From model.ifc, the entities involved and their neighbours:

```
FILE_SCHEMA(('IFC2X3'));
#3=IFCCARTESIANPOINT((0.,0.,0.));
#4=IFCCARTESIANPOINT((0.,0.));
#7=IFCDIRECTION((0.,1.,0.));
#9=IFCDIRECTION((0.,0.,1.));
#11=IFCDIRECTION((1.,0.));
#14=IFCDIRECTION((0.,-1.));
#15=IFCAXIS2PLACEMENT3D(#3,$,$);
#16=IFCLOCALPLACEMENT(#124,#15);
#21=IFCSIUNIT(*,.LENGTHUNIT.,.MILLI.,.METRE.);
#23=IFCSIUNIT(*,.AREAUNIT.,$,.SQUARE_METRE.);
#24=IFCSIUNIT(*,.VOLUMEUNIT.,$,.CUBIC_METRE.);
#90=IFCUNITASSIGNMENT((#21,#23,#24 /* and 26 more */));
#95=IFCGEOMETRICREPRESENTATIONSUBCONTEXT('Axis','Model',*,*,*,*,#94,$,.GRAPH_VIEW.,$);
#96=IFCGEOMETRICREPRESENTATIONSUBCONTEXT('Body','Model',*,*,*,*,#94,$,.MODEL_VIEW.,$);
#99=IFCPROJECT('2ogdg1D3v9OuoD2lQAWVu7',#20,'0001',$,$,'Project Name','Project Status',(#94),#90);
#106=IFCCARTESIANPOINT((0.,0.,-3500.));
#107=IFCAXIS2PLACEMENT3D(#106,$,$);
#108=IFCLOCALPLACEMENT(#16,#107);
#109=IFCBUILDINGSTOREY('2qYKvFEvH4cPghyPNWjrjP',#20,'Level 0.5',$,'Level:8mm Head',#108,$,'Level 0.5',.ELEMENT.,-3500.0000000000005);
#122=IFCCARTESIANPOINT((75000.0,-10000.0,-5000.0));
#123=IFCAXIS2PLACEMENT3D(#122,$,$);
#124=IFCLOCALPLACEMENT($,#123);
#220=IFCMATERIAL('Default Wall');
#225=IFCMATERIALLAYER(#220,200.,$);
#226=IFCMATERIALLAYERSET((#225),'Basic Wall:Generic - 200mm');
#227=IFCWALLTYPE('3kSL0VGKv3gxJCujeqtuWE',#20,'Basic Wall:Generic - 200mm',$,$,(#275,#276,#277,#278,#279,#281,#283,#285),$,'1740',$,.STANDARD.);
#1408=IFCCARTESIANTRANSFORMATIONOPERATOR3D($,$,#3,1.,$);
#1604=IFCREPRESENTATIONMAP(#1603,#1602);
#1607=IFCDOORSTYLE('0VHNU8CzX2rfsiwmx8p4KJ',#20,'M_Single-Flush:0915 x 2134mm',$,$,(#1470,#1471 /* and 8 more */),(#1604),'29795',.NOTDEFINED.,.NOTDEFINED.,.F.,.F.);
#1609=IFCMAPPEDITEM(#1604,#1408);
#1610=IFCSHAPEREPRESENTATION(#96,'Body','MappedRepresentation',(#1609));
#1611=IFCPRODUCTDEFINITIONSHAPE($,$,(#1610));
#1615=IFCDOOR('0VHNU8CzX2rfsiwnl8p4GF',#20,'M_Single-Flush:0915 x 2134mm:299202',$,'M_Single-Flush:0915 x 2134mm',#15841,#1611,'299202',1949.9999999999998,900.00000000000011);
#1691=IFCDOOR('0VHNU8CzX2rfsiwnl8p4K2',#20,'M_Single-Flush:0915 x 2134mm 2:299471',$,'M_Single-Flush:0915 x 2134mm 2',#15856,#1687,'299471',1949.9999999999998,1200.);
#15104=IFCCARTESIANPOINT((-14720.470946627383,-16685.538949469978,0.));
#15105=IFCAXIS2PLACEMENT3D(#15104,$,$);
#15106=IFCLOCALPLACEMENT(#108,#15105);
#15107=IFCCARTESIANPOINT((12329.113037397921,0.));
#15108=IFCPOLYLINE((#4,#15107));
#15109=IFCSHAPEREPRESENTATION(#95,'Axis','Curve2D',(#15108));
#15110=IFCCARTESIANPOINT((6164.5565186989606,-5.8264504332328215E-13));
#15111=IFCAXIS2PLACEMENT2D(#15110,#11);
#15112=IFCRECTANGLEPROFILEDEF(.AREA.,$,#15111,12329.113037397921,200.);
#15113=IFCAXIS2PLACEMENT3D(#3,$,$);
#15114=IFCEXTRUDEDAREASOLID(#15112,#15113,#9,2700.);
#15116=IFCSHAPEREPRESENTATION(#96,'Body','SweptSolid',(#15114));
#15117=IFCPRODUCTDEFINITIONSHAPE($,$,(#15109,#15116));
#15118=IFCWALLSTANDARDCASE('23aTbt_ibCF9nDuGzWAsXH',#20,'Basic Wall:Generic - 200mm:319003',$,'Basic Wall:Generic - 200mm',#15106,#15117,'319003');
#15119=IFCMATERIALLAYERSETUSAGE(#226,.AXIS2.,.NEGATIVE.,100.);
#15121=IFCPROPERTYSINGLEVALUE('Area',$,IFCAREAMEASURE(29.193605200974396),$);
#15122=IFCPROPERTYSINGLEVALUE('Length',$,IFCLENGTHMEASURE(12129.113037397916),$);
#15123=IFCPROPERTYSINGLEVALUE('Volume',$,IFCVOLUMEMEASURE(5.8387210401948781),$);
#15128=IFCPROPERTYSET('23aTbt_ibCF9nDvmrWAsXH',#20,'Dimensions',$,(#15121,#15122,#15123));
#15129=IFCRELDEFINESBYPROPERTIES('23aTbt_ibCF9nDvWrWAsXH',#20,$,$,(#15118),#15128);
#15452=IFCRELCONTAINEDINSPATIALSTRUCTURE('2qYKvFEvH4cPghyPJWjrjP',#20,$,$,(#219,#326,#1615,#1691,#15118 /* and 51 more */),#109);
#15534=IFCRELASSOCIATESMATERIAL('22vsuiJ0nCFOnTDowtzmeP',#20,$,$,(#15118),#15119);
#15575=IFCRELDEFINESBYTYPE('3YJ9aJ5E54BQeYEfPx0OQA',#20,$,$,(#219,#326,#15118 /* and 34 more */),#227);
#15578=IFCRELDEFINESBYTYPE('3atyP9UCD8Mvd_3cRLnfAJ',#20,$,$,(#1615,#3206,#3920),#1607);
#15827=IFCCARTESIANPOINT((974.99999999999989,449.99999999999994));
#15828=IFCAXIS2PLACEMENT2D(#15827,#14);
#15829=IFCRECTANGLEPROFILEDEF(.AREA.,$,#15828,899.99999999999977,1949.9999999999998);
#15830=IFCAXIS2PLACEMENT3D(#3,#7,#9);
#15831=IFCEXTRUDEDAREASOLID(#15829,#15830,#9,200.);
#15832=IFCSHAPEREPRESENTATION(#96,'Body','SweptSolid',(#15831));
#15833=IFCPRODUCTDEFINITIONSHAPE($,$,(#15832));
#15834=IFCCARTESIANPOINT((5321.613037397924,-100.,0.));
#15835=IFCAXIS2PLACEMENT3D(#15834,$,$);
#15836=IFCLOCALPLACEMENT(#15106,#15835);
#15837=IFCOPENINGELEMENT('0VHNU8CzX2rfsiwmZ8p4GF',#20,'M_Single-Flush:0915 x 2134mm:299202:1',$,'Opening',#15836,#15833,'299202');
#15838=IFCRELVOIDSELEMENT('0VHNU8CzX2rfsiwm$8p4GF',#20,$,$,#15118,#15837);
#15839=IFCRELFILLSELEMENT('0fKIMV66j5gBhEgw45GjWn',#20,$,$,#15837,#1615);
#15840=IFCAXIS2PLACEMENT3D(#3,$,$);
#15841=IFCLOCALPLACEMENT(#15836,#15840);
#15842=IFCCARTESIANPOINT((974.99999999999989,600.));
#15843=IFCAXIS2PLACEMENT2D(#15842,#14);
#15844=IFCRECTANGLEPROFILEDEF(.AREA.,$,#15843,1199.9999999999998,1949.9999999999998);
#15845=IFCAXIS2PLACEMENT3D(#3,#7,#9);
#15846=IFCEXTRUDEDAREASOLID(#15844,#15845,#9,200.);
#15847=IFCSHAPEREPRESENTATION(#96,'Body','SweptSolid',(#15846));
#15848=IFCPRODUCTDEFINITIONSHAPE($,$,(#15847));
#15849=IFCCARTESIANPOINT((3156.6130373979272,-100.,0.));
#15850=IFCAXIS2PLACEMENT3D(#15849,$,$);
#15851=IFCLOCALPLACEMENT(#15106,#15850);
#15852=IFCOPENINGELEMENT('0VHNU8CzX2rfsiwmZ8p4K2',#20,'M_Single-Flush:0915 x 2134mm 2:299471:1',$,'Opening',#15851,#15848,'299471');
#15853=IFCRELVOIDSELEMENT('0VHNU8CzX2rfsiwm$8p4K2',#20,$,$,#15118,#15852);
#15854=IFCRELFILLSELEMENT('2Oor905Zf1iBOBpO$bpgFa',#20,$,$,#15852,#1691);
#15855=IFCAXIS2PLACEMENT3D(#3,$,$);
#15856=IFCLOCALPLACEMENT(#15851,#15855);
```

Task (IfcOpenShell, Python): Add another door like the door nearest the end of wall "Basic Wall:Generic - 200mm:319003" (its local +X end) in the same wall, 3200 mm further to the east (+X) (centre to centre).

```python
import ifcopenshell
import ifcopenshell.api.feature
import ifcopenshell.api.geometry
import ifcopenshell.api.pset
import ifcopenshell.api.root
import ifcopenshell.geom
import ifcopenshell.util.element
import ifcopenshell.util.placement
import ifcopenshell.util.shape
import ifcopenshell.util.unit

model = ifcopenshell.open("model.ifc")
unit_scale = ifcopenshell.util.unit.calculate_unit_scale(model)
area_scale = ifcopenshell.util.unit.calculate_unit_scale(model, "AREAUNIT")
volume_scale = ifcopenshell.util.unit.calculate_unit_scale(model, "VOLUMEUNIT")
settings = ifcopenshell.geom.settings()


def volume(element):
    """Net volume in cubic metres, openings subtracted."""
    shape = ifcopenshell.geom.create_shape(settings, element)
    return ifcopenshell.util.shape.get_volume(shape.geometry)


def reuse_history(source, copy):
    """copy_class also copies each property set's owner history, people and application; keep the originals."""
    for rel in copy.IsDefinedBy:
        if rel.is_a("IfcRelDefinesByProperties") and (history := rel.RelatingPropertyDefinition.OwnerHistory):
            rel.RelatingPropertyDefinition.OwnerHistory = source.OwnerHistory
            ifcopenshell.util.element.remove_deep2(model, history)


door = model.by_guid("0VHNU8CzX2rfsiwnl8p4GF")
opening = door.FillsVoids[0].RelatingOpeningElement
wall = opening.VoidsElements[0].RelatingBuildingElement
before = volume(wall)
shift = ifcopenshell.util.placement.get_local_placement(wall.ObjectPlacement)[:3, 0] * 3.2 / unit_scale

# copy_class copies the void relationship, type, container and properties, but no geometry.
new_opening = ifcopenshell.api.root.copy_class(model, product=opening)
new_opening.Representation = ifcopenshell.util.element.copy_deep(
    model, opening.Representation, exclude=["IfcGeometricRepresentationContext", "IfcRepresentationMap"]
)
new_opening.Name = "M_Single-Flush:0915 x 2134mm"
new_opening.Tag = None
new_door = ifcopenshell.api.root.copy_class(model, product=door)
new_door.Representation = ifcopenshell.util.element.copy_deep(
    model, door.Representation, exclude=["IfcGeometricRepresentationContext", "IfcRepresentationMap"]
)
new_door.Name = "M_Single-Flush:0915 x 2134mm"
new_door.Tag = None
reuse_history(door, new_door)
fills = ifcopenshell.api.feature.add_filling(model, opening=new_opening, element=new_door)
fills.OwnerHistory = new_door.OwnerHistory  # required in IFC2X3

for old, new in ((opening, new_opening), (door, new_door)):
    matrix = ifcopenshell.util.placement.get_local_placement(old.ObjectPlacement)
    matrix[:3, 3] += shift
    ifcopenshell.api.geometry.edit_object_placement(model, product=new, matrix=matrix, is_si=False)

after = volume(wall)
thickness = 0.2  # wall thickness in metres

# Update the wall's stored quantities.
pset = model.by_id(ifcopenshell.util.element.get_pset(wall, "Dimensions", should_inherit=False)["id"])
ifcopenshell.api.pset.edit_pset(model, pset=pset, properties={
    "Area": model.create_entity("IfcAreaMeasure", after / thickness / area_scale),
    "Volume": model.create_entity("IfcVolumeMeasure", after / volume_scale),
})

print(f"wall volume {before:.3f} -> {after:.3f} m3")

model.write("model-out.ifc")
```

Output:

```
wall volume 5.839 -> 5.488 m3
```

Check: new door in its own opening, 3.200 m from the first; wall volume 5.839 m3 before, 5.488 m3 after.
